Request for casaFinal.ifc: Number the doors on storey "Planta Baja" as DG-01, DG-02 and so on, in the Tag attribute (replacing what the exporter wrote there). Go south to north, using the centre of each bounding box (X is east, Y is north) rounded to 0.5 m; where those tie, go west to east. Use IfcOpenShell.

First a look at what the model holds.

```python
import ifcopenshell
import ifcopenshell.util.element
import ifcopenshell.util.placement

model = ifcopenshell.open("casaFinal.ifc")
print(model.schema)
storey = next(s for s in model.by_type("IfcBuildingStorey") if s.Name == "Planta Baja")
doors = [e for e in ifcopenshell.util.element.get_decomposition(storey) if e.is_a("IfcDoor")]
for e in sorted(doors, key=lambda e: e.id()):
    origin = ifcopenshell.util.placement.get_local_placement(e.ObjectPlacement)[:3, 3]
    print(e.id(), e.Tag, e.Name, origin.round(2) + 0.0, sep=" | ")
```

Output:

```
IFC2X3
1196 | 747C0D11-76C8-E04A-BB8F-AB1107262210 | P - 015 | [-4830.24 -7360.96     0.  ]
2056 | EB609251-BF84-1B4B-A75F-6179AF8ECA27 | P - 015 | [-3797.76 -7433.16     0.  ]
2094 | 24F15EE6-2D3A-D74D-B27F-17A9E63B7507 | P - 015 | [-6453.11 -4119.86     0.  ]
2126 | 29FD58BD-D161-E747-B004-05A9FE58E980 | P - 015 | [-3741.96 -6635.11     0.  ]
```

```python
import ifcopenshell
import ifcopenshell.geom
import ifcopenshell.util.element
import ifcopenshell.util.shape

model = ifcopenshell.open("casaFinal.ifc")
settings = ifcopenshell.geom.settings()
settings.set("use-world-coords", True)


def centre(element):
    shape = ifcopenshell.geom.create_shape(settings, element)
    return ifcopenshell.util.shape.get_bbox_centroid(shape.geometry)


storey = next(s for s in model.by_type("IfcBuildingStorey") if s.Name == "Planta Baja")
doors = [e for e in ifcopenshell.util.element.get_decomposition(storey) if e.is_a("IfcDoor")]

# Insertion points can sit at a corner or the storey origin, so sort by the geometry (in metres).
centres = {e: centre(e) for e in doors}
doors.sort(key=lambda e: (round(centres[e][1] / 0.5), centres[e][0]))

for i, e in enumerate(doors, start=1):
    number = f"DG-{i:02d}"
    e.Tag = number
    print(e.id(), number)

model.write("casaFinal_rev.ifc")
```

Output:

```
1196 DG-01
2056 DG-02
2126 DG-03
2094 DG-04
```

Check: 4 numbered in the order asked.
